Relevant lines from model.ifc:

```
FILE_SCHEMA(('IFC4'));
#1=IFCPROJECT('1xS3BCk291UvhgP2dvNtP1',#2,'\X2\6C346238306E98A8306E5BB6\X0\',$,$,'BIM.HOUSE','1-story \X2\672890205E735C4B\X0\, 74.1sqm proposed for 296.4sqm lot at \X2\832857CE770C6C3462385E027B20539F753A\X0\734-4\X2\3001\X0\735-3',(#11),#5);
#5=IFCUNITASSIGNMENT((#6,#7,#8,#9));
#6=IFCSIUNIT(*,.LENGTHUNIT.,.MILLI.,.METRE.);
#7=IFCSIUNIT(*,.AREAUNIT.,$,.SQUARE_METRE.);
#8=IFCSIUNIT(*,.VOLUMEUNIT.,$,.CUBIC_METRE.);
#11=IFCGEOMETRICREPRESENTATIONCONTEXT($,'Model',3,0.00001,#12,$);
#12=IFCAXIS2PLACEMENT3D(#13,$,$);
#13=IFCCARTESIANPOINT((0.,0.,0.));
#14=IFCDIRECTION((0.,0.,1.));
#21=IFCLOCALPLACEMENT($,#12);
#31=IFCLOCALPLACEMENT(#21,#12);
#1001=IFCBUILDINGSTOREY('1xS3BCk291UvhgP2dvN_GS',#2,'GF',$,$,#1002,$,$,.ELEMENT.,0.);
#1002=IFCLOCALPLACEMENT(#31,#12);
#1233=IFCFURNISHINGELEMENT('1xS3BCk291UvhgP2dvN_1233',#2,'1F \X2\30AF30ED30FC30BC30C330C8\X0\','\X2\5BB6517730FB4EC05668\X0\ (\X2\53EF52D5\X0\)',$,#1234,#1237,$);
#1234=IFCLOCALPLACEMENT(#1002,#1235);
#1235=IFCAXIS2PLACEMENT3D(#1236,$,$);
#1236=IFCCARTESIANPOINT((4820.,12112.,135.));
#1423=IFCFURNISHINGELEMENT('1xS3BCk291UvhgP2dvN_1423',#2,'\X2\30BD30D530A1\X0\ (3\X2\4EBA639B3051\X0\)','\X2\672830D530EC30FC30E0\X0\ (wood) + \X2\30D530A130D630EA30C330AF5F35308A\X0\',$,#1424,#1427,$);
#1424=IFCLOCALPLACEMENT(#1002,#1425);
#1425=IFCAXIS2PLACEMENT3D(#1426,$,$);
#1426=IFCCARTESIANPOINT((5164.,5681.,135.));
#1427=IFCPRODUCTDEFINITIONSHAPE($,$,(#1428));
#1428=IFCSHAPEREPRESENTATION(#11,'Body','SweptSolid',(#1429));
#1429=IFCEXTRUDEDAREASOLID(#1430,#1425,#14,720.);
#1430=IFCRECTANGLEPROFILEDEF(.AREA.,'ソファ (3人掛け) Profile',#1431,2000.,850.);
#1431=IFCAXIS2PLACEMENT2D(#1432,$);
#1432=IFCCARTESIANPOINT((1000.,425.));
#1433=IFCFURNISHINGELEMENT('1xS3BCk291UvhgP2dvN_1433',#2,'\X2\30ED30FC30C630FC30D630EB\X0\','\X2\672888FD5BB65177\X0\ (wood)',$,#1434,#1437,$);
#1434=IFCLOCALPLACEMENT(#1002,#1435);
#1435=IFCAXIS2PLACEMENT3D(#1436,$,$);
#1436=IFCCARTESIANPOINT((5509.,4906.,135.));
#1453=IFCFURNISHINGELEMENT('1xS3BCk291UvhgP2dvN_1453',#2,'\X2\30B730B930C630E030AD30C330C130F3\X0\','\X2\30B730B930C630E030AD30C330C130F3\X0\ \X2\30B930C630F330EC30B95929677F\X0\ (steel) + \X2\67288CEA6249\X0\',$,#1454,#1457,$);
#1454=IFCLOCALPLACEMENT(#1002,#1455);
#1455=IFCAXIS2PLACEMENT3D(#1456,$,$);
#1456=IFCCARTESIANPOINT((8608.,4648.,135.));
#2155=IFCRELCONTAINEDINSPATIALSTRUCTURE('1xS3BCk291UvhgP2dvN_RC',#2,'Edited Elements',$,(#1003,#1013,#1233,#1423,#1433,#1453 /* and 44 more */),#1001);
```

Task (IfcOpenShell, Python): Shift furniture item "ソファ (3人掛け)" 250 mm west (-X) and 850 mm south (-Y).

```python
import ifcopenshell
import ifcopenshell.api.geometry
import ifcopenshell.util.placement

model = ifcopenshell.open("model.ifc")

item = model.by_guid("1xS3BCk291UvhgP2dvN_1423")
matrix = ifcopenshell.util.placement.get_local_placement(item.ObjectPlacement)
matrix[0, 3] -= 250.0
matrix[1, 3] -= 850.0
ifcopenshell.api.geometry.edit_object_placement(model, product=item, matrix=matrix, is_si=False)

print(ifcopenshell.util.placement.get_local_placement(item.ObjectPlacement).round(3) + 0.0)

model.write("model-out.ifc")
```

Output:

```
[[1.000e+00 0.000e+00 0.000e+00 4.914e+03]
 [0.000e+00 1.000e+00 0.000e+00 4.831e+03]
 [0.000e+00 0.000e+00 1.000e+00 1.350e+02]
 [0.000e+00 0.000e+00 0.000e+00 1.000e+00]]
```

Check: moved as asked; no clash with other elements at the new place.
